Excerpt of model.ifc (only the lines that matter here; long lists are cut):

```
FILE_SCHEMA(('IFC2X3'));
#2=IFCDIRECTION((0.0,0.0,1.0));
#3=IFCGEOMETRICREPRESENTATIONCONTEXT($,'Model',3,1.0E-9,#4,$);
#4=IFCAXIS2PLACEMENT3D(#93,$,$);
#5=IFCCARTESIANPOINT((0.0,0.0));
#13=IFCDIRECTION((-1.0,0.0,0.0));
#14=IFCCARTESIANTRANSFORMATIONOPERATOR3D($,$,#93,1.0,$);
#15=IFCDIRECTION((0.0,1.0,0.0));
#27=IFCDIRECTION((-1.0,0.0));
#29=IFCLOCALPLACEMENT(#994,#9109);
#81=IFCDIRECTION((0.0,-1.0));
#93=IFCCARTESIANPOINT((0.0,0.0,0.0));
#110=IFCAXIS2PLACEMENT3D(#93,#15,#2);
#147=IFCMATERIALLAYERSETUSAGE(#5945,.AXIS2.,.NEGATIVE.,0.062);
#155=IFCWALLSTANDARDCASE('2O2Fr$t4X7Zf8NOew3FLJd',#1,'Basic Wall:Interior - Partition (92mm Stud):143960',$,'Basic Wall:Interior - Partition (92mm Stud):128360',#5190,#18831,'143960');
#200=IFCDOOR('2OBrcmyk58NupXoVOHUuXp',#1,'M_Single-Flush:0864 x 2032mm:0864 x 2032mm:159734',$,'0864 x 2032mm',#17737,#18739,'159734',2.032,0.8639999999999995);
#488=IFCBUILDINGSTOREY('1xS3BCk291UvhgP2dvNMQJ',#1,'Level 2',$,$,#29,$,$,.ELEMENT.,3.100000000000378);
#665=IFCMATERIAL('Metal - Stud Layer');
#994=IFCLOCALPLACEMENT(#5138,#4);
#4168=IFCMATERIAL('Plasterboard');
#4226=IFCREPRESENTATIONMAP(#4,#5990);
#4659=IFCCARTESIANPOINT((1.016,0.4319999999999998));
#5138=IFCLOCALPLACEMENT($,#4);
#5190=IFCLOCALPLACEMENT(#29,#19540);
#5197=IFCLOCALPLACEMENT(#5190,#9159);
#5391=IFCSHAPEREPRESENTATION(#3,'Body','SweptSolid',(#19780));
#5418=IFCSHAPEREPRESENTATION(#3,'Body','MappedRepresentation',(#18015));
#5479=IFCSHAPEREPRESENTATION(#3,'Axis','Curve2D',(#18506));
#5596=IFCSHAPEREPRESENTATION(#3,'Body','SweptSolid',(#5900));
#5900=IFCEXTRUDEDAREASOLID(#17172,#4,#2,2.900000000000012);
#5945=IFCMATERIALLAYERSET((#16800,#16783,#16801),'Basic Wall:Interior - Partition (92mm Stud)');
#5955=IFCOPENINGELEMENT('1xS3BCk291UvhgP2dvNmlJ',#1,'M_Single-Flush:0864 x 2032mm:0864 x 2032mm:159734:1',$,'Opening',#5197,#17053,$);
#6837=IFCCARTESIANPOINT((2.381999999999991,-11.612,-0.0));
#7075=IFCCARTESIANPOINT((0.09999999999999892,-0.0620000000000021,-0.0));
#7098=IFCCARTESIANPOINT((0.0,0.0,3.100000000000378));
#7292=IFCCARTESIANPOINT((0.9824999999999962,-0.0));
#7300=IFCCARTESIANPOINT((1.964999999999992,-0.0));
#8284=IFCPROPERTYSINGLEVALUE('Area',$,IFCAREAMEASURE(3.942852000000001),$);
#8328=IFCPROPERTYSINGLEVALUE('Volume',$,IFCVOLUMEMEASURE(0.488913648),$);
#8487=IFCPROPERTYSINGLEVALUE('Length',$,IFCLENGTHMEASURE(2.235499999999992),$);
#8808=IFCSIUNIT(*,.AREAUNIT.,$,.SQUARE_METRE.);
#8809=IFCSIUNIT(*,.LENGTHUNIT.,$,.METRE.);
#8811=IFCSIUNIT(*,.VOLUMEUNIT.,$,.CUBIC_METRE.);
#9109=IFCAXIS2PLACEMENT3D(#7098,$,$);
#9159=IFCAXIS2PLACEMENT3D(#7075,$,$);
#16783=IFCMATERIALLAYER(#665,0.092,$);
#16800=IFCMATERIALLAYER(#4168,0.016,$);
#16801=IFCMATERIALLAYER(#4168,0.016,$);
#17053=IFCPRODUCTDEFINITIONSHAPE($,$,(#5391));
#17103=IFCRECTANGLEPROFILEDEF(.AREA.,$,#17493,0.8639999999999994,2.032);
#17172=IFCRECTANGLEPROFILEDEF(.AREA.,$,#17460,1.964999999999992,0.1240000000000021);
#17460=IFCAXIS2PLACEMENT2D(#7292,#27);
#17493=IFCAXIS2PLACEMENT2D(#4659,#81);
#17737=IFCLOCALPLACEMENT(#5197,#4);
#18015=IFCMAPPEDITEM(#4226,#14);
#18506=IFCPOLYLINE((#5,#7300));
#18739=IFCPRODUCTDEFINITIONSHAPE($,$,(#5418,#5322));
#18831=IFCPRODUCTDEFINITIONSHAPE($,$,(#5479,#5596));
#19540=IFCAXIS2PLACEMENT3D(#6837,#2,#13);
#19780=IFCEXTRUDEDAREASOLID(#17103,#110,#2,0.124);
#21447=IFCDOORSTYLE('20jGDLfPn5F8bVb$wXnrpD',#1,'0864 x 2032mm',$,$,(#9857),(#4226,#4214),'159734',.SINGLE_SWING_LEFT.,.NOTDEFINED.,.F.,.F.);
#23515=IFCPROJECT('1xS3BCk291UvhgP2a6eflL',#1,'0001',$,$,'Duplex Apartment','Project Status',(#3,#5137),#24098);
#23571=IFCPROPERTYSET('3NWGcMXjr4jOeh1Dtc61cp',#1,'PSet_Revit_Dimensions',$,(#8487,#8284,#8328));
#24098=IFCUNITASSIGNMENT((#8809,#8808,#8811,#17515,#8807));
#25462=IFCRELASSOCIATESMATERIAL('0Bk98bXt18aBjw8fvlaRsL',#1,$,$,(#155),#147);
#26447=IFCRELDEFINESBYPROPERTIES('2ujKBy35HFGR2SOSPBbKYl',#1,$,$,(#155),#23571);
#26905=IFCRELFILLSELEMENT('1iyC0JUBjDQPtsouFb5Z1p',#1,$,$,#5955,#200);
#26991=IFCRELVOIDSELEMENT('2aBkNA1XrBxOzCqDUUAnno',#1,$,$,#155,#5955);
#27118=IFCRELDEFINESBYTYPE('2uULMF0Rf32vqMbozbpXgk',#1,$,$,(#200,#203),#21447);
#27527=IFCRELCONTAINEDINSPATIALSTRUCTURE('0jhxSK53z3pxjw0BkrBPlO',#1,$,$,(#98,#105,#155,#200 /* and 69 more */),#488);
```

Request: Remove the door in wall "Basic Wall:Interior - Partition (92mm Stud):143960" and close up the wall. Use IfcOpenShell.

```python
import ifcopenshell
import ifcopenshell.api.feature
import ifcopenshell.api.pset
import ifcopenshell.api.root
import ifcopenshell.geom
import ifcopenshell.util.element
import ifcopenshell.util.shape
import ifcopenshell.util.unit

model = ifcopenshell.open("model.ifc")
area_scale = ifcopenshell.util.unit.calculate_unit_scale(model, "AREAUNIT")
volume_scale = ifcopenshell.util.unit.calculate_unit_scale(model, "VOLUMEUNIT")
settings = ifcopenshell.geom.settings()


def volume(element):
    """Net volume in cubic metres, openings subtracted."""
    shape = ifcopenshell.geom.create_shape(settings, element)
    return ifcopenshell.util.shape.get_volume(shape.geometry)


door = model.by_id(200)
opening = door.FillsVoids[0].RelatingOpeningElement
wall = opening.VoidsElements[0].RelatingBuildingElement
before = volume(wall)

ifcopenshell.api.root.remove_product(model, product=door)
ifcopenshell.api.feature.remove_feature(model, feature=opening)

after = volume(wall)
thickness = 0.124  # wall thickness in metres

# Update the wall's stored quantities.
pset = model.by_id(ifcopenshell.util.element.get_pset(wall, "PSet_Revit_Dimensions", should_inherit=False)["id"])
ifcopenshell.api.pset.edit_pset(model, pset=pset, properties={
    "Area": model.create_entity("IfcAreaMeasure", after / thickness / area_scale),
    "Volume": model.create_entity("IfcVolumeMeasure", after / volume_scale),
})

print(f"wall volume {before:.3f} -> {after:.3f} m3")

model.write("model_updated.ifc")
```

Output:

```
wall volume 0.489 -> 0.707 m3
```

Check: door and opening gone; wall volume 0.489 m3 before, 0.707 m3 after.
